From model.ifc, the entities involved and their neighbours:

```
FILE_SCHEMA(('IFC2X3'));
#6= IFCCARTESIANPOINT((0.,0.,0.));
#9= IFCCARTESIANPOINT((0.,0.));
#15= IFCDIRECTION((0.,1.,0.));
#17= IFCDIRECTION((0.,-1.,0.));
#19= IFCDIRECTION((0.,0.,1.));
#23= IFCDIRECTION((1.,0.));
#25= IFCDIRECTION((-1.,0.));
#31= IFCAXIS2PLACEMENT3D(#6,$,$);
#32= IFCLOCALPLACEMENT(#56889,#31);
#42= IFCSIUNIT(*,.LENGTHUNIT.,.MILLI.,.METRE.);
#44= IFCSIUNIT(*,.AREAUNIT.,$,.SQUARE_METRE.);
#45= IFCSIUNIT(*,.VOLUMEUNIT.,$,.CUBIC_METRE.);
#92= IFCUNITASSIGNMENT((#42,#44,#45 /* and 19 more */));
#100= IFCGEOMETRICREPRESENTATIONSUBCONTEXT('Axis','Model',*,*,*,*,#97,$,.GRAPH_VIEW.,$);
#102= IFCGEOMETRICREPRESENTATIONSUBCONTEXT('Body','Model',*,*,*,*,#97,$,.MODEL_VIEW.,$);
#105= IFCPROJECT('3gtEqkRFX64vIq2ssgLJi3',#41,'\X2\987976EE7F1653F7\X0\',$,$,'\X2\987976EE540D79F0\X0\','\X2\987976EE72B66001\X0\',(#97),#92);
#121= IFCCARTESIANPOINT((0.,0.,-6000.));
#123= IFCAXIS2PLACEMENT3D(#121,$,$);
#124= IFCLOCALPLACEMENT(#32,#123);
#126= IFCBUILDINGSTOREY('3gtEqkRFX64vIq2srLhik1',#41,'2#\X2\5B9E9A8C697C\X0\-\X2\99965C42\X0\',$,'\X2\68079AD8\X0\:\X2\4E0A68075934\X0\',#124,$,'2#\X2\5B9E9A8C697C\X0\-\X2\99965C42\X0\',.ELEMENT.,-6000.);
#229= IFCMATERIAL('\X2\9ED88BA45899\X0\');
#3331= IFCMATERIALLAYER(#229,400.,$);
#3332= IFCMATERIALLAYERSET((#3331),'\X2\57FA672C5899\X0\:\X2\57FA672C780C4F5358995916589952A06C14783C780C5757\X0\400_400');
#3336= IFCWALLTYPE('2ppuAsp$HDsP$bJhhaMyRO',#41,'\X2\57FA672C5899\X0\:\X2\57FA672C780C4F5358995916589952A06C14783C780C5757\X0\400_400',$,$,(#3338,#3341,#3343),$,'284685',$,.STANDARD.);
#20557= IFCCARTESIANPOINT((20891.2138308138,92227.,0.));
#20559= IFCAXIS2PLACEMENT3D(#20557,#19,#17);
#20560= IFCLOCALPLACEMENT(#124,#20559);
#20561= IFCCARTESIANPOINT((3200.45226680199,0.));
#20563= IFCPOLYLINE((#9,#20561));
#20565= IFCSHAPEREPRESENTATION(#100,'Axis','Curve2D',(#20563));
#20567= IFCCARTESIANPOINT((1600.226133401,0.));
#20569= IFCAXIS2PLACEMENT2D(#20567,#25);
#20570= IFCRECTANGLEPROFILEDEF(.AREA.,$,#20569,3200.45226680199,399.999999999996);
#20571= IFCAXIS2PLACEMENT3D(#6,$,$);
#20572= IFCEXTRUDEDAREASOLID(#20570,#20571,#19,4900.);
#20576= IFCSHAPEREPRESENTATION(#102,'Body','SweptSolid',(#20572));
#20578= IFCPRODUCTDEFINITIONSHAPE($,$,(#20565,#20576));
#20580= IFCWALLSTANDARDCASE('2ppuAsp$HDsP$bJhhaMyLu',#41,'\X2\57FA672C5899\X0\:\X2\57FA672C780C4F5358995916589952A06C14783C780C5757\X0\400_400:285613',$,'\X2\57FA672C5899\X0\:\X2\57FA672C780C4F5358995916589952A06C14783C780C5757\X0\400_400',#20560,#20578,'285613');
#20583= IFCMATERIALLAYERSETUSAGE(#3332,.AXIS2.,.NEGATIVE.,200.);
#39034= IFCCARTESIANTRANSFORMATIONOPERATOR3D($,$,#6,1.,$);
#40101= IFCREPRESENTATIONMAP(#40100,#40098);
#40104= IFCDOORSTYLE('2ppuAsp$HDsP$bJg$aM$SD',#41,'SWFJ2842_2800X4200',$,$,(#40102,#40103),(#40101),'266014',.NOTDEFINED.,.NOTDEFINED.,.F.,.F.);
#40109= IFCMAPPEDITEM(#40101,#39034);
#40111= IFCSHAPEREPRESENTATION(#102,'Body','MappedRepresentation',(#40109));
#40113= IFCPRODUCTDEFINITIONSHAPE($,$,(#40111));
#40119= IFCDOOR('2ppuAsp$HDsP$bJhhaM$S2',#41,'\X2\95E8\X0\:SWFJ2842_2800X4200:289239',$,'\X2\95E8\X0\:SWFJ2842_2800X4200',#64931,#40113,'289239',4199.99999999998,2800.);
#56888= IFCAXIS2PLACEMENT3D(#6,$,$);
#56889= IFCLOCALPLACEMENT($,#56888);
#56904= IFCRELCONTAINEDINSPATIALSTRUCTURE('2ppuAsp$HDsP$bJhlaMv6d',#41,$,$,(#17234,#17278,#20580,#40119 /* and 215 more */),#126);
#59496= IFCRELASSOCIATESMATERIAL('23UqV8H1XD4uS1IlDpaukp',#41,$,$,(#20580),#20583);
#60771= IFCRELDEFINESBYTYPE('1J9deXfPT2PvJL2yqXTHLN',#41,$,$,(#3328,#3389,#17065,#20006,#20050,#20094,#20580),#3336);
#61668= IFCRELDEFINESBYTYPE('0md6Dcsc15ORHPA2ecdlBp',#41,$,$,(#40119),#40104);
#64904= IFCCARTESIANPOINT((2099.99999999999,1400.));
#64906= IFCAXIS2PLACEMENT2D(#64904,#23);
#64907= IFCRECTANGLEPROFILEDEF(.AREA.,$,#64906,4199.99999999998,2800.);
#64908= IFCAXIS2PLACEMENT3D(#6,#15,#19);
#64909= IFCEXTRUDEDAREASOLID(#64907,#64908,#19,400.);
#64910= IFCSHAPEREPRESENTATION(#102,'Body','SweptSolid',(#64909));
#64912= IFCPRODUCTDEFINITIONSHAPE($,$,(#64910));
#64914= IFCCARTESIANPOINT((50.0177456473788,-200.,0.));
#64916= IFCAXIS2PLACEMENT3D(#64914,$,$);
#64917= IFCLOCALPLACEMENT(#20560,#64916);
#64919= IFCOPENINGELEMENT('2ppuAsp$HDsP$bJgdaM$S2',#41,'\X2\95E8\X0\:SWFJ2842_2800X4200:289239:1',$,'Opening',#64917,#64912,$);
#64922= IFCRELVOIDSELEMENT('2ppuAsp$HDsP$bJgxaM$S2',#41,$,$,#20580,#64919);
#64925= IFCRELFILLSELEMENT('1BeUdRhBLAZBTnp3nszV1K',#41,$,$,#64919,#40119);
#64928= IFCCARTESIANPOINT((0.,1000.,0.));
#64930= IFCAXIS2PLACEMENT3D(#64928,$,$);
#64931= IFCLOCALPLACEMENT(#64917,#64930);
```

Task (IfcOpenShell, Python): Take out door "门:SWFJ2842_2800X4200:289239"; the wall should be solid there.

```python
import ifcopenshell
import ifcopenshell.api.feature
import ifcopenshell.api.root
import ifcopenshell.geom
import ifcopenshell.util.shape

model = ifcopenshell.open("model.ifc")
settings = ifcopenshell.geom.settings()


def volume(element):
    """Net volume in cubic metres, openings subtracted."""
    shape = ifcopenshell.geom.create_shape(settings, element)
    return ifcopenshell.util.shape.get_volume(shape.geometry)


door = model.by_guid("2ppuAsp$HDsP$bJhhaM$S2")
opening = door.FillsVoids[0].RelatingOpeningElement
wall = opening.VoidsElements[0].RelatingBuildingElement
before = volume(wall)

ifcopenshell.api.root.remove_product(model, product=door)
ifcopenshell.api.feature.remove_feature(model, feature=opening)

after = volume(wall)

print(f"wall volume {before:.3f} -> {after:.3f} m3")

model.write("model_rev.ifc")
```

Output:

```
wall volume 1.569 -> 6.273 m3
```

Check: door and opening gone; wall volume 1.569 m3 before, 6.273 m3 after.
